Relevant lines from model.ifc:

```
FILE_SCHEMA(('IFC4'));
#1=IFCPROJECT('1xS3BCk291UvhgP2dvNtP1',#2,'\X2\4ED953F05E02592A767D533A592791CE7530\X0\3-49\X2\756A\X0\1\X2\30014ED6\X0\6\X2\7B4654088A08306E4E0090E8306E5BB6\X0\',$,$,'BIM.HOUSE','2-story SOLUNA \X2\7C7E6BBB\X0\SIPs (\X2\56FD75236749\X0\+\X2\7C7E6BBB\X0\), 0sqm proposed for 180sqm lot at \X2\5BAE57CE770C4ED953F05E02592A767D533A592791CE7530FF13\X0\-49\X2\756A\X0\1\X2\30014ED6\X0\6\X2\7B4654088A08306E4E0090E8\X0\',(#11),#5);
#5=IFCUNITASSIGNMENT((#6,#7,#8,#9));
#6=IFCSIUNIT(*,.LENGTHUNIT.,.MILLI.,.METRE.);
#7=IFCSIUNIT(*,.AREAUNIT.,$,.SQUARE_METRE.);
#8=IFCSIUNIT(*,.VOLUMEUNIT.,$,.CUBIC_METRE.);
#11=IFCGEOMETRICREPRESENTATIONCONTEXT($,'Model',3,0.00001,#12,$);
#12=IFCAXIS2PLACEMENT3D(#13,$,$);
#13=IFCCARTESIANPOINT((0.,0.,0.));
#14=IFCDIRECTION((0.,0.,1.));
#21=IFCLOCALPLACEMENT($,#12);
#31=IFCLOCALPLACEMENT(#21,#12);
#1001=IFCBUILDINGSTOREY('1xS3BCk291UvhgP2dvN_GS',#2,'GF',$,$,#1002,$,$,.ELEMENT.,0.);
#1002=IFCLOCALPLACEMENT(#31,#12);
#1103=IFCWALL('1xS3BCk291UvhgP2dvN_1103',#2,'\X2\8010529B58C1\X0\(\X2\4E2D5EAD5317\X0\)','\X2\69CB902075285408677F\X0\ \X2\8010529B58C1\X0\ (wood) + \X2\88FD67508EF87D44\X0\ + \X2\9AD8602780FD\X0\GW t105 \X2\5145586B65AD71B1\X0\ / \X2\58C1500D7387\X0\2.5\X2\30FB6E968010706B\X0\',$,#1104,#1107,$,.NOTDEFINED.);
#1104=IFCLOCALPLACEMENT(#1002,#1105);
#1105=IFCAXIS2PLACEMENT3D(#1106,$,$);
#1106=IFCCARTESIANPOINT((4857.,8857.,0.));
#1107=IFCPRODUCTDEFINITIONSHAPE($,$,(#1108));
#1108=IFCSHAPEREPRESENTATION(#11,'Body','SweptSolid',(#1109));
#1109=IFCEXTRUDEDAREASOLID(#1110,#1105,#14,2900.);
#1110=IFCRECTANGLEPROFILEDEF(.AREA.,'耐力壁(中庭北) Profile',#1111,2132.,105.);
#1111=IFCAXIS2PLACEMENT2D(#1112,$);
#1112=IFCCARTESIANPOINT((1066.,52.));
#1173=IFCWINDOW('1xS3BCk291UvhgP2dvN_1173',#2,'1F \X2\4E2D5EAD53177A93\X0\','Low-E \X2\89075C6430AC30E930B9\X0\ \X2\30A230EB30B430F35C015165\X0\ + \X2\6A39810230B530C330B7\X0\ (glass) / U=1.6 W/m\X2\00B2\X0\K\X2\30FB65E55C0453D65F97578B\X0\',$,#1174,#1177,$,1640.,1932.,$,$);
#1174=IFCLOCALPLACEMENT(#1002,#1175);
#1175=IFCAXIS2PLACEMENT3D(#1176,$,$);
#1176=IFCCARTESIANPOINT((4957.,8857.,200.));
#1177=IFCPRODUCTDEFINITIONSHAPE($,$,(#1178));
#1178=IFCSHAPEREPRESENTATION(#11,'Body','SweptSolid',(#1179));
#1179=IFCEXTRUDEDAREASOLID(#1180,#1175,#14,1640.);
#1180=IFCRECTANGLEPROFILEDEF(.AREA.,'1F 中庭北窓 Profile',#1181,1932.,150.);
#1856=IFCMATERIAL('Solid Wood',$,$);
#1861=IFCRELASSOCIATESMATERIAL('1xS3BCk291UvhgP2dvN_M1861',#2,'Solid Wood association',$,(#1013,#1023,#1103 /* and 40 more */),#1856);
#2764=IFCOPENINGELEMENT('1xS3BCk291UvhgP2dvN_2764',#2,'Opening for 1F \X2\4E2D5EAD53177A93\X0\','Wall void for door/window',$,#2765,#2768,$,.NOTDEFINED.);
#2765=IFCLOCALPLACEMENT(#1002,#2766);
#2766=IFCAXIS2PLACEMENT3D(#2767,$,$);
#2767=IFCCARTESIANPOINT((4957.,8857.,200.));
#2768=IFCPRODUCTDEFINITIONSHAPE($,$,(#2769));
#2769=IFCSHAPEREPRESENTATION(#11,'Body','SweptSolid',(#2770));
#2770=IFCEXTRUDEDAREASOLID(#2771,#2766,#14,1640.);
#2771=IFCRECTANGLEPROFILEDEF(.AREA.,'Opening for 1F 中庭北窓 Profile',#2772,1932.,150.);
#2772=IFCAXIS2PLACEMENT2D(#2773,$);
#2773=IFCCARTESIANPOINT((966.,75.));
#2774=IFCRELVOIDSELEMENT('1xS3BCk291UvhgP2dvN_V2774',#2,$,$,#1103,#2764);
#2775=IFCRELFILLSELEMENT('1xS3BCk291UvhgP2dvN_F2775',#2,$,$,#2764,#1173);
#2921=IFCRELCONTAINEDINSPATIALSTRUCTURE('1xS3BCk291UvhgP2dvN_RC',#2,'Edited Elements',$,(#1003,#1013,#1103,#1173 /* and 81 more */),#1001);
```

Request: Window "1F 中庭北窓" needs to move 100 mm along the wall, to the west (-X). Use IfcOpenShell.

```python
import ifcopenshell
import ifcopenshell.api.geometry
import ifcopenshell.util.placement

model = ifcopenshell.open("model.ifc")

window = model.by_guid("1xS3BCk291UvhgP2dvN_1173")
opening = window.FillsVoids[0].RelatingOpeningElement
wall = opening.VoidsElements[0].RelatingBuildingElement

wall_matrix = ifcopenshell.util.placement.get_local_placement(wall.ObjectPlacement)
shift = wall_matrix[:3, 0] * -100.0
before = ifcopenshell.util.placement.get_local_placement(window.ObjectPlacement)[:3, 3].copy()

# The window is not placed relative to its opening, so move both.
for product in (opening, window):
    matrix = ifcopenshell.util.placement.get_local_placement(product.ObjectPlacement)
    matrix[:3, 3] += shift
    ifcopenshell.api.geometry.edit_object_placement(model, product=product, matrix=matrix, is_si=False)

after = ifcopenshell.util.placement.get_local_placement(window.ObjectPlacement)[:3, 3]
print("window moved by", (after - before).round(3) + 0.0)

model.write("model_edited.ifc")
```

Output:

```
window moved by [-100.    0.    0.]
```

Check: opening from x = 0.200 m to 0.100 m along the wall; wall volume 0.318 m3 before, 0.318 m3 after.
